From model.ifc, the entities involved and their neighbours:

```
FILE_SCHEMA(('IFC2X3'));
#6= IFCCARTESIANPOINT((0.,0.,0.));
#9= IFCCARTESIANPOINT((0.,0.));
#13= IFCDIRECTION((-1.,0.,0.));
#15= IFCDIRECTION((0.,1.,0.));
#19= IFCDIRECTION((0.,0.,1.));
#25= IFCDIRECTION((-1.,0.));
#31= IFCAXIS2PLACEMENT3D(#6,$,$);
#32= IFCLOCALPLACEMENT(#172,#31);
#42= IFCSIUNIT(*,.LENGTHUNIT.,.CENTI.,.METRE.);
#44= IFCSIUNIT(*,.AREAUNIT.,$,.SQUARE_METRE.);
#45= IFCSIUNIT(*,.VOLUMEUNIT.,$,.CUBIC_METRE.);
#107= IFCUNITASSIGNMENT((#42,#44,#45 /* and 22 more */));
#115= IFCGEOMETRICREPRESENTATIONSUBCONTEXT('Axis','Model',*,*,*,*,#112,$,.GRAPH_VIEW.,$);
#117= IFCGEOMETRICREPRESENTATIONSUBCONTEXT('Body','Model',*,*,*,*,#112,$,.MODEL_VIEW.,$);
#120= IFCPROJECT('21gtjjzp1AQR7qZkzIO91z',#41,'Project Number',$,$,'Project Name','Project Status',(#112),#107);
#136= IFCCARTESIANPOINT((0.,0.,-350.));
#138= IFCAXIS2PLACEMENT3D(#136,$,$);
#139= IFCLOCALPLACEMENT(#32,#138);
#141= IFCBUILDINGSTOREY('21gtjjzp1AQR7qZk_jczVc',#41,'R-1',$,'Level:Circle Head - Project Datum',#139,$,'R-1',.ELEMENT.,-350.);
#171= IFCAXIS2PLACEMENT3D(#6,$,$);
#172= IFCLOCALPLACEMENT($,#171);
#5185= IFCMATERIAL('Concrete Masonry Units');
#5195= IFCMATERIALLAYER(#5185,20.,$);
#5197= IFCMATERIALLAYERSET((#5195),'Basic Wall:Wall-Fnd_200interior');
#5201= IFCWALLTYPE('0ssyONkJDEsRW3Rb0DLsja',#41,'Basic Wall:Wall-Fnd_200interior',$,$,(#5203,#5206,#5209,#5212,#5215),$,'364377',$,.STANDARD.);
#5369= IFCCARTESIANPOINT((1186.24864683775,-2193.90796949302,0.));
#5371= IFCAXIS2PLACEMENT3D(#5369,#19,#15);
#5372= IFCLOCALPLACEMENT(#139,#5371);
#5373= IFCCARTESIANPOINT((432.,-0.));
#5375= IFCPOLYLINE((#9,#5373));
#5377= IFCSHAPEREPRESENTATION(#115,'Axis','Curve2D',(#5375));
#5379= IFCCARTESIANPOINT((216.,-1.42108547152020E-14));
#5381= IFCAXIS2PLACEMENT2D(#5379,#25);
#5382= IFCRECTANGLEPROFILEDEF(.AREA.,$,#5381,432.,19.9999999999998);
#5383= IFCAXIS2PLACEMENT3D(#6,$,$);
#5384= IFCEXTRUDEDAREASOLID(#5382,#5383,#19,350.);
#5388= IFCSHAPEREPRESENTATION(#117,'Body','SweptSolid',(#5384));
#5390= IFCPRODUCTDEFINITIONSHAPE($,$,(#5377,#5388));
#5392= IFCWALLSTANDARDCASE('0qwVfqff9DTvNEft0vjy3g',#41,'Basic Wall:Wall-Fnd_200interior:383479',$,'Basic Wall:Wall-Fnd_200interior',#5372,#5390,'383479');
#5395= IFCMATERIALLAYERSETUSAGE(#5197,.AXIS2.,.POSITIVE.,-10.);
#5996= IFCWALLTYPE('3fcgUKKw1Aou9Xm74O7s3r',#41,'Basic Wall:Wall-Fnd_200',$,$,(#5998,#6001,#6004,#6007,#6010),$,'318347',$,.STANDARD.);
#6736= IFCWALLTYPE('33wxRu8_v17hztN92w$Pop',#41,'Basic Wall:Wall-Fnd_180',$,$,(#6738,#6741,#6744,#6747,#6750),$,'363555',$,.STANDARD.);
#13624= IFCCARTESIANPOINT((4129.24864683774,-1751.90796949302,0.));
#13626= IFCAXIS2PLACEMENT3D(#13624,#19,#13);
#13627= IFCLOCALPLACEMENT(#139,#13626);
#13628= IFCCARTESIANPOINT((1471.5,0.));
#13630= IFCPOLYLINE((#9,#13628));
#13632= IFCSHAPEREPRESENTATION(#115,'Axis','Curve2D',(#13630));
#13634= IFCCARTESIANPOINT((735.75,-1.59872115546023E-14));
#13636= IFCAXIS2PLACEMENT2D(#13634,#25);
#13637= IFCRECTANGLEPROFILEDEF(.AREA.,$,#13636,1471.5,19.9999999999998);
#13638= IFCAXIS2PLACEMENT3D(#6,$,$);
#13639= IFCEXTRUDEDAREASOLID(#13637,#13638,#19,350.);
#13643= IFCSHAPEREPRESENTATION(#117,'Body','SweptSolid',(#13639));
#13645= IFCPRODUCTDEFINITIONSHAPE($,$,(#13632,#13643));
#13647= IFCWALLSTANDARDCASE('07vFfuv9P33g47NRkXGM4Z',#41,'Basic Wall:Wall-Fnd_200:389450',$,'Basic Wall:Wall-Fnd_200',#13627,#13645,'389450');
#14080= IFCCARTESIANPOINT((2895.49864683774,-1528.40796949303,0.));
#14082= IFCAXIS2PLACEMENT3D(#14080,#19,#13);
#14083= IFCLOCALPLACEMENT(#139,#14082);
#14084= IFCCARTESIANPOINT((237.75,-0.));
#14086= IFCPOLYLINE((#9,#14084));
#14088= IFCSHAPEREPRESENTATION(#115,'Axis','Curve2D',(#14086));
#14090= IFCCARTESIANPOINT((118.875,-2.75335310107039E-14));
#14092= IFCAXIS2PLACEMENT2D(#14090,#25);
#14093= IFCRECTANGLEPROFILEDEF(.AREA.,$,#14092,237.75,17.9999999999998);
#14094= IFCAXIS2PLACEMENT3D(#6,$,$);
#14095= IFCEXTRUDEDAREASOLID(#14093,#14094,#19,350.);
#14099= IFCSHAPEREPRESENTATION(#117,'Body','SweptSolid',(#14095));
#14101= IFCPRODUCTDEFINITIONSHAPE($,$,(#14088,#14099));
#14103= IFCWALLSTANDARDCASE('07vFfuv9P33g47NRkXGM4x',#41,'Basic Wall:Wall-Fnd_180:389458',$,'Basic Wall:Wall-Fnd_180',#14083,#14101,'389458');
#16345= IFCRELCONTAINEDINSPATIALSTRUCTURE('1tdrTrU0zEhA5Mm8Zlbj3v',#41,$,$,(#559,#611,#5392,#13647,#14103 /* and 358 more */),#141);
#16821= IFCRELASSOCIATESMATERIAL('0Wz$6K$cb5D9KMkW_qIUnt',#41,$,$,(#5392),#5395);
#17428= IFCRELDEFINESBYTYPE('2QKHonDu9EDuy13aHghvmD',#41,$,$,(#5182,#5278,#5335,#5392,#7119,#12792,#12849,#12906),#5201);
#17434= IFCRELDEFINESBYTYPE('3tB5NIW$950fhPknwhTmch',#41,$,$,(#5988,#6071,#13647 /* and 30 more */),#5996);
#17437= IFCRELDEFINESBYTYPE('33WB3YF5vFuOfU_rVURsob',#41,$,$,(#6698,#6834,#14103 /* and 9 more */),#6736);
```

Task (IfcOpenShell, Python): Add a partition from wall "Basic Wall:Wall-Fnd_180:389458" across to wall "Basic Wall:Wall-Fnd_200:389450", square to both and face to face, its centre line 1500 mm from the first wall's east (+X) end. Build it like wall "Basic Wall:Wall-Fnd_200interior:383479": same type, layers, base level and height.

```python
import numpy as np
import ifcopenshell
import ifcopenshell.api.geometry
import ifcopenshell.api.material
import ifcopenshell.api.pset
import ifcopenshell.api.root
import ifcopenshell.api.spatial
import ifcopenshell.api.type
import ifcopenshell.geom
import ifcopenshell.util.element
import ifcopenshell.util.placement
import ifcopenshell.util.representation
import ifcopenshell.util.shape
import ifcopenshell.util.unit

model = ifcopenshell.open("model.ifc")
unit_scale = ifcopenshell.util.unit.calculate_unit_scale(model)
settings = ifcopenshell.geom.settings()
settings.set("use-world-coords", True)

start_wall = model.by_id(14103)
end_wall = model.by_id(13647)
like = model.by_guid("0qwVfqff9DTvNEft0vjy3g")
matrix = ifcopenshell.util.placement.get_local_placement(start_wall.ObjectPlacement)
matrix[:3, 3] *= unit_scale


def extent(element):
    """Bounding box in the first wall's axes, in metres."""
    shape = ifcopenshell.geom.create_shape(settings, element)
    points = (ifcopenshell.util.shape.get_vertices(shape.geometry) - matrix[:3, 3]) @ matrix[:3, :3]
    return points.min(axis=0), points.max(axis=0)


y_start = extent(start_wall)[1][1]
y_end = extent(end_wall)[0][1]
like_min, like_max = extent(like)
length, height = float(abs(y_end - y_start)), float(like_max[2] - like_min[2])
layer_set = ifcopenshell.util.element.get_material(like, should_skip_usage=True)
thickness = sum(layer.LayerThickness for layer in layer_set.MaterialLayers) * unit_scale

wall = ifcopenshell.api.root.create_entity(model, ifc_class="IfcWallStandardCase", name="New partition")
storey = ifcopenshell.util.element.get_container(like)
ifcopenshell.api.spatial.assign_container(model, products=[wall], relating_structure=storey)
ifcopenshell.api.type.assign_type(
    model, related_objects=[wall], relating_type=ifcopenshell.util.element.get_type(like), should_map_representations=False
)
rel = ifcopenshell.api.material.assign_material(
    model, products=[wall], type="IfcMaterialLayerSetUsage", material=layer_set
)
rel.RelatingMaterial.OffsetFromReferenceLine = -thickness / 2 / unit_scale
pset = ifcopenshell.api.pset.add_pset(model, product=wall, name="Pset_WallCommon")
ifcopenshell.api.pset.edit_pset(model, pset=pset, properties={"IsExternal": False, "LoadBearing": False})

# The axis runs down the middle of the wall.
axis = ifcopenshell.api.geometry.add_axis_representation(
    model, context=ifcopenshell.util.representation.get_context(model, "Model", "Axis"), axis=[(0.0, 0.0), (length, 0.0)]
)
body = ifcopenshell.api.geometry.add_wall_representation(
    model,
    context=ifcopenshell.util.representation.get_context(model, "Model", "Body", "MODEL_VIEW"),
    length=length,
    height=height,
    thickness=thickness,
    offset=-thickness / 2,
)
for representation in (axis, body):
    ifcopenshell.api.geometry.assign_representation(model, product=wall, representation=representation)

placement = matrix @ ifcopenshell.util.placement.rotation(90, "Z")
placement[:, 3] = matrix @ np.array([extent(start_wall)[0][0] + 1.5, y_start, like_min[2], 1.0])
ifcopenshell.api.geometry.edit_object_placement(model, product=wall, matrix=placement)

print(f"partition {length:.3f} m long, {height:.3f} m high, {thickness:.3f} m thick")

model.write("model-out.ifc")
```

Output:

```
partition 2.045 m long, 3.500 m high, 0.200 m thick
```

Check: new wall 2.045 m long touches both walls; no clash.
